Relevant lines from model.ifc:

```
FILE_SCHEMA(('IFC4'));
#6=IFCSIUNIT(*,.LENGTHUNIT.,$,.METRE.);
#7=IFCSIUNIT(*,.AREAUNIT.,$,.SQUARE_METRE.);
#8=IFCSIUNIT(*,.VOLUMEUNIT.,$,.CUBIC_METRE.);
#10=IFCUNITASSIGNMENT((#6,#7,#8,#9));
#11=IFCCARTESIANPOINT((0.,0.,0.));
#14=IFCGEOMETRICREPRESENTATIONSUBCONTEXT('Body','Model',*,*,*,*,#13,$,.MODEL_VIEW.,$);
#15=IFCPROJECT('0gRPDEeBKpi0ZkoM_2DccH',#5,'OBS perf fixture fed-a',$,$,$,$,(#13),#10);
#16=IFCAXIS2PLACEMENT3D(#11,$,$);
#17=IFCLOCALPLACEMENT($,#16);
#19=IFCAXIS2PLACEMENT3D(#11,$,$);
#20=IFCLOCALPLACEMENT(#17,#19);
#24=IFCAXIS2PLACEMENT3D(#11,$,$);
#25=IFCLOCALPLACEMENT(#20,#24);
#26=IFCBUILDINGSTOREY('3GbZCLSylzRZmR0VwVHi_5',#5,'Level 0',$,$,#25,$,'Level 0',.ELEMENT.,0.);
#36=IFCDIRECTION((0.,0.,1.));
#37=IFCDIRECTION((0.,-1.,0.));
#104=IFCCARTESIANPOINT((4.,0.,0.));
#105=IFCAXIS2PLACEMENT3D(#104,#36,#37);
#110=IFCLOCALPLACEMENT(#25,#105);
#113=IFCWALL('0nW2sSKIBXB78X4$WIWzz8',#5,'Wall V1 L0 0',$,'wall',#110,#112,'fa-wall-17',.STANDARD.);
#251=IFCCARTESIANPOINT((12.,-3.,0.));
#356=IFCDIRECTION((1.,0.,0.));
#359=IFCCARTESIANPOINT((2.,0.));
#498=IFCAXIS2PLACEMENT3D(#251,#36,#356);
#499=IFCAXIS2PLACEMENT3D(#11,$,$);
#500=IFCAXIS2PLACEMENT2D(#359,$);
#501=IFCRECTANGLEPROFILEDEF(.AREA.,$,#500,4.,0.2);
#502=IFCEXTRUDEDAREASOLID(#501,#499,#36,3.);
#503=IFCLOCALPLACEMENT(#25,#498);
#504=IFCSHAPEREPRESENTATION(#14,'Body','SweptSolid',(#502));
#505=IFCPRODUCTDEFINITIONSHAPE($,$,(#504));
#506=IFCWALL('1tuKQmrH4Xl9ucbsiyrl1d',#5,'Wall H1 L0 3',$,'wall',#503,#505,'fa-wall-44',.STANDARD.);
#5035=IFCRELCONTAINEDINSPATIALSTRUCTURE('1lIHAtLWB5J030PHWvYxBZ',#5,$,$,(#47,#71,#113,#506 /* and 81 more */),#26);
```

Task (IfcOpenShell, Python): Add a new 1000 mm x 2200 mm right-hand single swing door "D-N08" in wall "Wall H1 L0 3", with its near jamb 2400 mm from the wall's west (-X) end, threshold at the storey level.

```python
import numpy as np
import ifcopenshell
import ifcopenshell.api.feature
import ifcopenshell.api.geometry
import ifcopenshell.api.root
import ifcopenshell.api.spatial
import ifcopenshell.geom
import ifcopenshell.util.element
import ifcopenshell.util.placement
import ifcopenshell.util.representation
import ifcopenshell.util.shape
import ifcopenshell.util.unit

model = ifcopenshell.open("model.ifc")
unit_scale = ifcopenshell.util.unit.calculate_unit_scale(model)
settings = ifcopenshell.geom.settings()


def volume(element):
    """Net volume in cubic metres, openings subtracted."""
    shape = ifcopenshell.geom.create_shape(settings, element)
    return ifcopenshell.util.shape.get_volume(shape.geometry)


wall = model.by_guid("1tuKQmrH4Xl9ucbsiyrl1d")
storey = ifcopenshell.util.element.get_container(wall, ifc_class="IfcBuildingStorey")
context = ifcopenshell.util.representation.get_context(model, "Model", "Body", "MODEL_VIEW")
before = volume(wall)

width, height, from_end, sill = 1, 2.2, 2.4, 0.0  # metres

# The wall runs along its own X axis, and the end named is its -X end.
wall_shape = ifcopenshell.geom.create_shape(settings, wall)
x, y, z = ifcopenshell.util.shape.get_vertices(wall_shape.geometry).T
start = x.min() + from_end
face, thickness = float(y.min()), float(y.max() - y.min())
wall_matrix = ifcopenshell.util.placement.get_local_placement(wall.ObjectPlacement)
level = ifcopenshell.util.placement.get_local_placement(storey.ObjectPlacement)[2, 3]


def in_wall(x, y):
    """Placement at x, y metres in the wall's axes, at sill height."""
    matrix = wall_matrix.copy()
    matrix[:, 3] = wall_matrix @ np.array([x / unit_scale, y / unit_scale, 0.0, 1.0])
    matrix[2, 3] = level + sill / unit_scale
    return matrix


# Opening: a box that overshoots both wall faces by 50 mm.
opening = ifcopenshell.api.root.create_entity(model, ifc_class="IfcOpeningElement", predefined_type="OPENING")
box = ifcopenshell.api.geometry.add_wall_representation(
    model, context=context, length=width, height=height, thickness=thickness + 0.1
)
ifcopenshell.api.geometry.assign_representation(model, product=opening, representation=box)
ifcopenshell.api.geometry.edit_object_placement(model, product=opening, matrix=in_wall(start, face - 0.05), is_si=False)
ifcopenshell.api.feature.add_feature(model, feature=opening, element=wall)

door = ifcopenshell.api.root.create_entity(model, ifc_class="IfcDoor", name="D-N08", predefined_type="DOOR")
door.OverallWidth, door.OverallHeight = width / unit_scale, height / unit_scale
door.OperationType = "SINGLE_SWING_RIGHT"
body = ifcopenshell.api.geometry.add_door_representation(
    model,
    context=context,
    overall_width=door.OverallWidth,
    overall_height=door.OverallHeight,
    operation_type="SINGLE_SWING_RIGHT",
    lining_properties={"LiningDepth": thickness / unit_scale, "ThresholdDepth": thickness / unit_scale},
)
ifcopenshell.api.geometry.assign_representation(model, product=door, representation=body)
ifcopenshell.api.spatial.assign_container(model, products=[door], relating_structure=storey)
ifcopenshell.api.feature.add_filling(model, opening=opening, element=door)

# The lining spans the wall, so the door starts at the wall face.
ifcopenshell.api.geometry.edit_object_placement(model, product=door, matrix=in_wall(start, face), is_si=False)

after = volume(wall)

print(f"wall volume {before:.3f} -> {after:.3f} m3")

model.write("model_updated.ifc")
```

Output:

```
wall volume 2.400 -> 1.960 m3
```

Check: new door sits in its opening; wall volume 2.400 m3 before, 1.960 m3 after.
